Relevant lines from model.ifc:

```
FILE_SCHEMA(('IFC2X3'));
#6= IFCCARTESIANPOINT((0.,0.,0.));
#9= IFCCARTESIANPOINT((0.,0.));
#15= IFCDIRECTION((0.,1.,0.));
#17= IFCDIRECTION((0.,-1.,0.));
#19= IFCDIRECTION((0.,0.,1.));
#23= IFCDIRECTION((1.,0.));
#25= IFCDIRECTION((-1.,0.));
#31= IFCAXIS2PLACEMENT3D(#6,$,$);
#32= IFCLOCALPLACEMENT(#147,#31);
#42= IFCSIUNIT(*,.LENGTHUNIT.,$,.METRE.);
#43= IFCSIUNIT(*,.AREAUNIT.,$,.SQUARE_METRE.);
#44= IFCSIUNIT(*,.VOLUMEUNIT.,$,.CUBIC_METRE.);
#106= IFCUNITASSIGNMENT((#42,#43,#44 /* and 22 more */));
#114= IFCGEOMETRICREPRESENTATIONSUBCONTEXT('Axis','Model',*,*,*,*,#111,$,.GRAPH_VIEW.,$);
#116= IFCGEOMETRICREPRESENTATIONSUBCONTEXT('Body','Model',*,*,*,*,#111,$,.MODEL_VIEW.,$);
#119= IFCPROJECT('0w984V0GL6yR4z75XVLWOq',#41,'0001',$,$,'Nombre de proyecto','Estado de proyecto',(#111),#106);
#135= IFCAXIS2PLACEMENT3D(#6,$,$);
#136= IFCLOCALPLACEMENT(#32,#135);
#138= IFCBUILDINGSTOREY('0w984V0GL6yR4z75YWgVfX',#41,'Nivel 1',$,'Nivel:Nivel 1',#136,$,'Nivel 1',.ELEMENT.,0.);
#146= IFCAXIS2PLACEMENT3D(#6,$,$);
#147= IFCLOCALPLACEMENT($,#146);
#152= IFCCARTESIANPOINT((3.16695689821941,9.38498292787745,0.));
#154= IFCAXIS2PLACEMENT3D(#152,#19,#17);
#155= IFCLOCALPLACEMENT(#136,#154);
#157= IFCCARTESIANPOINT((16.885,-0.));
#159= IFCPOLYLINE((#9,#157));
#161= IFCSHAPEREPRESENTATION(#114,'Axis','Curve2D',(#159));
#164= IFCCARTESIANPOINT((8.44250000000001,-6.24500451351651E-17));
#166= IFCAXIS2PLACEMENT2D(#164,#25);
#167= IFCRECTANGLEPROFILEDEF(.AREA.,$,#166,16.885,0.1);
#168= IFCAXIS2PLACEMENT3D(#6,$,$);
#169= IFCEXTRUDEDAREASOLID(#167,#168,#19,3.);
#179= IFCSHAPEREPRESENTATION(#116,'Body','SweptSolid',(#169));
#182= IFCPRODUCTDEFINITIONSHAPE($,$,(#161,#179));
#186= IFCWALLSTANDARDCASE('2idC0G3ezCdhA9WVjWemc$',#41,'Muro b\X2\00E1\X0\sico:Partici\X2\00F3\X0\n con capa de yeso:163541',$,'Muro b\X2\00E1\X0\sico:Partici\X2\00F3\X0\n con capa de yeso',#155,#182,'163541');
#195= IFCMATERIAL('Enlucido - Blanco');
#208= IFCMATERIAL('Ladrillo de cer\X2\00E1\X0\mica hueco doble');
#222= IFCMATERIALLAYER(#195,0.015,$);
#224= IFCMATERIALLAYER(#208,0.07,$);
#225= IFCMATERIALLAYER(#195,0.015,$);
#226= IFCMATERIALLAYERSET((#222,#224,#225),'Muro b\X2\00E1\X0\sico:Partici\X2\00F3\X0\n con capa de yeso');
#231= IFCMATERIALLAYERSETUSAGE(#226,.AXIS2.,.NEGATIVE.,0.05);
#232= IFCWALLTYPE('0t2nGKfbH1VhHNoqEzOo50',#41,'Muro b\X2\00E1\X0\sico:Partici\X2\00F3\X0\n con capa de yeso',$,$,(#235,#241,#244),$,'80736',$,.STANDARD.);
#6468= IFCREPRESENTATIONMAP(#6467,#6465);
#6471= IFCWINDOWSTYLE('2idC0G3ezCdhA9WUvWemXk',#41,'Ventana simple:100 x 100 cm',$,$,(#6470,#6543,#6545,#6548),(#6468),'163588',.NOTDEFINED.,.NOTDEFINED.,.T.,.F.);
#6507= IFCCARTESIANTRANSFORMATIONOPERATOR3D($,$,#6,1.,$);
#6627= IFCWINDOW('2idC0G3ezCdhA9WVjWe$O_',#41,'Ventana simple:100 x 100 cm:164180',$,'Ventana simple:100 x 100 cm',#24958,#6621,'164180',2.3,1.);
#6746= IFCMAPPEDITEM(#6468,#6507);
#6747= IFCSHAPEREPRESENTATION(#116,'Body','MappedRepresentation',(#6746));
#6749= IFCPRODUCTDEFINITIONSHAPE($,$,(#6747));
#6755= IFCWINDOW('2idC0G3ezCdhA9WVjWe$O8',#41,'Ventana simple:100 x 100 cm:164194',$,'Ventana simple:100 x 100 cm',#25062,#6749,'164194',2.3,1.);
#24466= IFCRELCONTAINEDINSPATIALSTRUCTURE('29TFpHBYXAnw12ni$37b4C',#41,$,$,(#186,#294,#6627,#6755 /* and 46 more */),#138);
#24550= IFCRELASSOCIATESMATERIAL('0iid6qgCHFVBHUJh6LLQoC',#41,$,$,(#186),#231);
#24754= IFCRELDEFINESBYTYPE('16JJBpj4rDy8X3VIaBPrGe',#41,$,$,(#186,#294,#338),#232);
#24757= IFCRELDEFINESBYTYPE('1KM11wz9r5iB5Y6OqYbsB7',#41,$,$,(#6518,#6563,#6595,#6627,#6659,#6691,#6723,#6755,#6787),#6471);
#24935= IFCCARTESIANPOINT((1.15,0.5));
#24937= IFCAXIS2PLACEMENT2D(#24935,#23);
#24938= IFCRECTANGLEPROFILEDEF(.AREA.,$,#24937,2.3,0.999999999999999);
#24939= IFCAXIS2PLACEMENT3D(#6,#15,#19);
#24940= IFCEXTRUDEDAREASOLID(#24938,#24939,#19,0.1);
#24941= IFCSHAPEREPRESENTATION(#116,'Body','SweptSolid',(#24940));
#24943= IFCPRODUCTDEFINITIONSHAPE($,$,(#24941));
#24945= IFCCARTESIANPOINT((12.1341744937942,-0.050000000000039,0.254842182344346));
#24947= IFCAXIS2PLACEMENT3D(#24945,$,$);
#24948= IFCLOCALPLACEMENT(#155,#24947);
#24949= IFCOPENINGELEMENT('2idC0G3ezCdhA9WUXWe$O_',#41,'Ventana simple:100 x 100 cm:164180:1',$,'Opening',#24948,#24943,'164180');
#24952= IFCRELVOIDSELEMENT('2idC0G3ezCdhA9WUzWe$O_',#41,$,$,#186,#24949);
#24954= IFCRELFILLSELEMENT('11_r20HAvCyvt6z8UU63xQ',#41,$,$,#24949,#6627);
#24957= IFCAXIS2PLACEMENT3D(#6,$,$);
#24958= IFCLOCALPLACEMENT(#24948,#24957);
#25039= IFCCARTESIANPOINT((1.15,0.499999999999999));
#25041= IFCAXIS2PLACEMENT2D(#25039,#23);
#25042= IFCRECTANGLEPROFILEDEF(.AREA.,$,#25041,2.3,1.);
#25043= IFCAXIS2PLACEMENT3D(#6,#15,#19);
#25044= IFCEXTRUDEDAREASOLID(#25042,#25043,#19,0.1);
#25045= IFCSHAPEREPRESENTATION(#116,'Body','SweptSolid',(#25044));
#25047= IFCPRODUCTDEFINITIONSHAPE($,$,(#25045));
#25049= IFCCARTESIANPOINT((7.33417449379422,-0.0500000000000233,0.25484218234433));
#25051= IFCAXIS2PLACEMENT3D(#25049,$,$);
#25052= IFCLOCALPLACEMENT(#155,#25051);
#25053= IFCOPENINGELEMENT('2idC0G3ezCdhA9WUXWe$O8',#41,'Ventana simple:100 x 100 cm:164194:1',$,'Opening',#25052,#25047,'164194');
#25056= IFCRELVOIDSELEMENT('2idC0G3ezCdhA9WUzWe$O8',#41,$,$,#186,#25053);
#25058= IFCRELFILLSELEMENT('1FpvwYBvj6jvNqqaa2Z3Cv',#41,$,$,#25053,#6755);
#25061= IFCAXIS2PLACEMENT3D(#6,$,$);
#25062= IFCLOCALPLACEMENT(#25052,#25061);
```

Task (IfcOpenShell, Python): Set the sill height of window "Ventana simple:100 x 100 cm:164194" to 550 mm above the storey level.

```python
import numpy as np
import ifcopenshell
import ifcopenshell.api.geometry
import ifcopenshell.geom
import ifcopenshell.util.element
import ifcopenshell.util.placement
import ifcopenshell.util.shape
import ifcopenshell.util.unit

model = ifcopenshell.open("model.ifc")
unit_scale = ifcopenshell.util.unit.calculate_unit_scale(model)

window = model.by_guid("2idC0G3ezCdhA9WVjWe$O8")
opening = window.FillsVoids[0].RelatingOpeningElement
storey = ifcopenshell.util.element.get_container(window, ifc_class="IfcBuildingStorey")
level = ifcopenshell.util.placement.get_local_placement(storey.ObjectPlacement)[2, 3]

# The opening's origin need not be at the sill, so measure its lowest point.
shape = ifcopenshell.geom.create_shape(ifcopenshell.geom.settings(), opening)
bottom = ifcopenshell.util.shape.get_shape_bottom_elevation(shape, shape.geometry) / unit_scale
dz = level + 0.55 / unit_scale - bottom

shift = np.array([0.0, 0.0, dz])
# The window is placed relative to its opening, so it follows when the opening moves.
matrix = ifcopenshell.util.placement.get_local_placement(opening.ObjectPlacement)
matrix[:3, 3] += shift
ifcopenshell.api.geometry.edit_object_placement(
    model, product=opening, matrix=matrix, is_si=False, should_transform_children=True
)

print(f"moved by {dz * unit_scale:+.3f} m")

model.write("model_edited.ifc")
```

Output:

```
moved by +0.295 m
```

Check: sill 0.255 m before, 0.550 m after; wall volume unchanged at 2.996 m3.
